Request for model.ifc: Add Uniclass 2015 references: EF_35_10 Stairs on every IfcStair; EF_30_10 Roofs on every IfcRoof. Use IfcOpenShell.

First a look at what the model holds.

```python
import ifcopenshell

model = ifcopenshell.open("model.ifc")
print(model.schema)
print("classifications:", [c.Name for c in model.by_type("IfcClassification")])
for ifc_class in ("IfcDoor", "IfcRoof", "IfcStair", "IfcWall", "IfcWindow"):
    print(ifc_class, len(model.by_type(ifc_class)))
```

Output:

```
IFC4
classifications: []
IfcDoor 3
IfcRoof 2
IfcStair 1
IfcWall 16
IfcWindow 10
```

```python
import ifcopenshell
import ifcopenshell.api.classification

model = ifcopenshell.open("model.ifc")

system = ifcopenshell.api.classification.add_classification(model, classification="Uniclass 2015")

codes = {
    "IfcStair": ("EF_35_10", "Stairs"),
    "IfcRoof": ("EF_30_10", "Roofs"),
}
for ifc_class, (code, name) in codes.items():
    products = model.by_type(ifc_class)
    ifcopenshell.api.classification.add_reference(
        model, products=products, classification=system, identification=code, name=name
    )
    print(code, len(products))

model.write("model_rev.ifc")
```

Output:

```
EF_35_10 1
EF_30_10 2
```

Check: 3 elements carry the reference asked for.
